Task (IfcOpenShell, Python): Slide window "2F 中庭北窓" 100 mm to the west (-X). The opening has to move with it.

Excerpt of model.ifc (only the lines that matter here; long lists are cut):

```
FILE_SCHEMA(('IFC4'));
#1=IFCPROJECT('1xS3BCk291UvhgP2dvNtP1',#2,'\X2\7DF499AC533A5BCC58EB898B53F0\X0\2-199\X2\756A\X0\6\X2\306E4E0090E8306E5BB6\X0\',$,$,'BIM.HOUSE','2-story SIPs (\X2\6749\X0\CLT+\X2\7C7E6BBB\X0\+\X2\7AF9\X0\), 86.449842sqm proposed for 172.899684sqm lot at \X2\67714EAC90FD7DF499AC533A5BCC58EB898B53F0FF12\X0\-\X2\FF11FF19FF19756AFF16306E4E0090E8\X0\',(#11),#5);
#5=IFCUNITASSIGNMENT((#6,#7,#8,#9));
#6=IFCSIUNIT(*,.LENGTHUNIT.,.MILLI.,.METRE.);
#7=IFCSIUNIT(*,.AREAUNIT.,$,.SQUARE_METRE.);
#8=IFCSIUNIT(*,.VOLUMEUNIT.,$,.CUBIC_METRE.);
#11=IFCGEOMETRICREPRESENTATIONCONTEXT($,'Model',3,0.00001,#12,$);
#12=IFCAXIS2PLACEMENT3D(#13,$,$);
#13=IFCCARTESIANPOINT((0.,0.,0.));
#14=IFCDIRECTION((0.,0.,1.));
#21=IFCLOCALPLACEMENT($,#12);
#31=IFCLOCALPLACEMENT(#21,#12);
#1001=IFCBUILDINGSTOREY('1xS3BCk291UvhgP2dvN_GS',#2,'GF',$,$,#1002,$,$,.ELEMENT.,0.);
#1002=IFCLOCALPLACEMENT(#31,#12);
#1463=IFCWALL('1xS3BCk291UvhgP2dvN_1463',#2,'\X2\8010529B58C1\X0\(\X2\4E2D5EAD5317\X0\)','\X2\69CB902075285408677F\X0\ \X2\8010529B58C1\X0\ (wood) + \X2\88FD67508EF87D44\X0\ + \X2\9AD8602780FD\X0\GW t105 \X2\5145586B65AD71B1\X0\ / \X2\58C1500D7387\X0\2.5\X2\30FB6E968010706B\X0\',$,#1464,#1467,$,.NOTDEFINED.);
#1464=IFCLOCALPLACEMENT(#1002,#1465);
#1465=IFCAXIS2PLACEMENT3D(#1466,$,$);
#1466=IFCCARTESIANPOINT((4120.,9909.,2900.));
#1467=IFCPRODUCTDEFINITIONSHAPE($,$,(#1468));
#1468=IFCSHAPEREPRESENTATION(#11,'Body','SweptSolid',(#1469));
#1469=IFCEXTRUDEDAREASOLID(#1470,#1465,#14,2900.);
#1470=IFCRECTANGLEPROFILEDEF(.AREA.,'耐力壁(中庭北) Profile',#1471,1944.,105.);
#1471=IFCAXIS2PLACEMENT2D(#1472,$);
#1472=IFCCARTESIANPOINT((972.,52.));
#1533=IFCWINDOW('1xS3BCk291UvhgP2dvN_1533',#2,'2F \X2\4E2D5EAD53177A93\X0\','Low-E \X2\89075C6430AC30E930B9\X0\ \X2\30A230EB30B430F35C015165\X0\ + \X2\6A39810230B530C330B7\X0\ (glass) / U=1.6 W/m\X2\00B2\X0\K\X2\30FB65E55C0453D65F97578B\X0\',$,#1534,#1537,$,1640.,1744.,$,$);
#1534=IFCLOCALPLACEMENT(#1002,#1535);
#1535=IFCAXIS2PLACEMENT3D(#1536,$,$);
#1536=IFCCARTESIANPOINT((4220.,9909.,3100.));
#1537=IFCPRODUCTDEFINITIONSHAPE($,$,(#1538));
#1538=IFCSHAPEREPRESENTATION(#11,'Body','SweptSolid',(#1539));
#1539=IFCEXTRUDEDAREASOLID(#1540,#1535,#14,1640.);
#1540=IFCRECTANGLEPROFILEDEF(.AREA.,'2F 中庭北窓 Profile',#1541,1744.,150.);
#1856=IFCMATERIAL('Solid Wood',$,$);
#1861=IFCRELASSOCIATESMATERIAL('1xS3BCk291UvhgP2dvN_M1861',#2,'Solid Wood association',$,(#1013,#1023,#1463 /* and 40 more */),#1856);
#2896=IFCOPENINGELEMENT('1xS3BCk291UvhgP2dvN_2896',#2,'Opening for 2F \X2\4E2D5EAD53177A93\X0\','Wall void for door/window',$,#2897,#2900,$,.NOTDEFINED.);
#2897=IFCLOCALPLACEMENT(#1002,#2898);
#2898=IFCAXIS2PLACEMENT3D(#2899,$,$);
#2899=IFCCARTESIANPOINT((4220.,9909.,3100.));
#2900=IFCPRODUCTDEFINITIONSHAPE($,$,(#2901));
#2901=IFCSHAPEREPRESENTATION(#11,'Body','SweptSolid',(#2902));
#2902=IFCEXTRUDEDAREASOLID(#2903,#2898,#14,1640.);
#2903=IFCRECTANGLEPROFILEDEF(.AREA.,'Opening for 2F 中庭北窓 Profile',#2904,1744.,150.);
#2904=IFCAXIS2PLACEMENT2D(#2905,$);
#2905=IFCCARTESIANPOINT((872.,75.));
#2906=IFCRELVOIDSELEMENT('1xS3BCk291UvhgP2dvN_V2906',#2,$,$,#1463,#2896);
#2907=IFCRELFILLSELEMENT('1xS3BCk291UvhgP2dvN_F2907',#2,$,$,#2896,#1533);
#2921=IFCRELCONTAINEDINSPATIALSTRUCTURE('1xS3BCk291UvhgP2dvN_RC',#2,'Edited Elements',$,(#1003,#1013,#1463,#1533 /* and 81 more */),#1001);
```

```python
import ifcopenshell
import ifcopenshell.api.geometry
import ifcopenshell.util.placement
import ifcopenshell.util.unit

model = ifcopenshell.open("model.ifc")
unit_scale = ifcopenshell.util.unit.calculate_unit_scale(model)

window = model.by_id(1533)
opening = window.FillsVoids[0].RelatingOpeningElement
wall = opening.VoidsElements[0].RelatingBuildingElement

wall_matrix = ifcopenshell.util.placement.get_local_placement(wall.ObjectPlacement)
shift = wall_matrix[:3, 0] * -0.1 / unit_scale
before = ifcopenshell.util.placement.get_local_placement(window.ObjectPlacement)[:3, 3].copy()

# The window is not placed relative to its opening, so move both.
for product in (opening, window):
    matrix = ifcopenshell.util.placement.get_local_placement(product.ObjectPlacement)
    matrix[:3, 3] += shift
    ifcopenshell.api.geometry.edit_object_placement(model, product=product, matrix=matrix, is_si=False)

after = ifcopenshell.util.placement.get_local_placement(window.ObjectPlacement)[:3, 3]
print("window moved by", (after - before).round(3) + 0.0)

model.write("model_rev.ifc")
```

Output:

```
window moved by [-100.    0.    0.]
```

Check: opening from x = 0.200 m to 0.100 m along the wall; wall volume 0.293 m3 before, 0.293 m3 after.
